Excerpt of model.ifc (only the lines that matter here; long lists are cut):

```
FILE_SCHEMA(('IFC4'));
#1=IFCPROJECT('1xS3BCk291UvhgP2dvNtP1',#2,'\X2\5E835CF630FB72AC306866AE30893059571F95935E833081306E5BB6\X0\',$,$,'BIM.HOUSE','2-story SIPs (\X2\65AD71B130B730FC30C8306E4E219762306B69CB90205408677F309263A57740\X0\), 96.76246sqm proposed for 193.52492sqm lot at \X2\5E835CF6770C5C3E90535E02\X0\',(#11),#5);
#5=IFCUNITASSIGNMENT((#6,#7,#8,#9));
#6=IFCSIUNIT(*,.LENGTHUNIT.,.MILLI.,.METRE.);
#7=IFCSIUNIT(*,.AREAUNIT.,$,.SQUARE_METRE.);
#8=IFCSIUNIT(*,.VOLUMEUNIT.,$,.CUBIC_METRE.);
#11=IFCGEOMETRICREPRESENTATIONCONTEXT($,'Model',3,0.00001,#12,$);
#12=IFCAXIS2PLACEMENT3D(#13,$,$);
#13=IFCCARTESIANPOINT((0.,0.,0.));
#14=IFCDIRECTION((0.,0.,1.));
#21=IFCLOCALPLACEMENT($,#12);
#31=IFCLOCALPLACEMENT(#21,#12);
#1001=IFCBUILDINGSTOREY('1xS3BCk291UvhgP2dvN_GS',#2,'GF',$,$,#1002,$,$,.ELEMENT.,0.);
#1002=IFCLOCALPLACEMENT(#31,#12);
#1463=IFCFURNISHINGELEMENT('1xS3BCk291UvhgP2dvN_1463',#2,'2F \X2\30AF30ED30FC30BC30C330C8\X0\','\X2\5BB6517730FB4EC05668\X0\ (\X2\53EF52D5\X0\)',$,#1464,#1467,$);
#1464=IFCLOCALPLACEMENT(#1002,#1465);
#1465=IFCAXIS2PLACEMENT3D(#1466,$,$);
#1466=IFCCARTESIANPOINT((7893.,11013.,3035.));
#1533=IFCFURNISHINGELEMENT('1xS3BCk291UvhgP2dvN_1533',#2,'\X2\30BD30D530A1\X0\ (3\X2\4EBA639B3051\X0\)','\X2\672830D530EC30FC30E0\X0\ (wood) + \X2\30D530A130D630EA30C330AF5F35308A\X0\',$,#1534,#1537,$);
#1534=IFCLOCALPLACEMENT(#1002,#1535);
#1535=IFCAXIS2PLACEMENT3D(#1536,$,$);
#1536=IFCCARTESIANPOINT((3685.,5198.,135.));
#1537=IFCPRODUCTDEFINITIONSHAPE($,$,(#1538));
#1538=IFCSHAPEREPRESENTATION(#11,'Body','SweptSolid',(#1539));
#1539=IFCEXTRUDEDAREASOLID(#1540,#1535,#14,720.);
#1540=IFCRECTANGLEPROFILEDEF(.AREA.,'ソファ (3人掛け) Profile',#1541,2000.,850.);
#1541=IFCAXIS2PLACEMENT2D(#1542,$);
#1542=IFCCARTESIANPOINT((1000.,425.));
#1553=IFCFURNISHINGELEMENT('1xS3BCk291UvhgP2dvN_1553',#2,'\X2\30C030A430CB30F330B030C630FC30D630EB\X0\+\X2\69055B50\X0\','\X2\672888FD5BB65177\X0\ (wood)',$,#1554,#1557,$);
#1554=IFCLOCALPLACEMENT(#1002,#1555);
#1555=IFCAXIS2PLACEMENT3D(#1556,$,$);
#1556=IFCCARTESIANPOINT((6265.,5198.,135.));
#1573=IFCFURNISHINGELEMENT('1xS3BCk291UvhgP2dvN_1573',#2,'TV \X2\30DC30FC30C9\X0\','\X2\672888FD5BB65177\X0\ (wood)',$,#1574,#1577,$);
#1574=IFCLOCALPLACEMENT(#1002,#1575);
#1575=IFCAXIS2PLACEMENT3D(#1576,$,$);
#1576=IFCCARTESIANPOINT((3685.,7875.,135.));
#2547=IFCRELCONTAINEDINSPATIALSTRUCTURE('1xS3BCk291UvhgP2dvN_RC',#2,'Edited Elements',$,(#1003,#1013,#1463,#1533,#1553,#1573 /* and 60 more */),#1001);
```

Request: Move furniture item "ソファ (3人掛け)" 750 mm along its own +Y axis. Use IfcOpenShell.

```python
import ifcopenshell
import ifcopenshell.api.geometry
import ifcopenshell.util.placement

model = ifcopenshell.open("model.ifc")

item = model.by_id(1533)
matrix = ifcopenshell.util.placement.get_local_placement(item.ObjectPlacement)
matrix[:3, 3] += matrix[:3, 1] * 750.0
ifcopenshell.api.geometry.edit_object_placement(model, product=item, matrix=matrix, is_si=False)

print(ifcopenshell.util.placement.get_local_placement(item.ObjectPlacement).round(3) + 0.0)

model.write("model_v2.ifc")
```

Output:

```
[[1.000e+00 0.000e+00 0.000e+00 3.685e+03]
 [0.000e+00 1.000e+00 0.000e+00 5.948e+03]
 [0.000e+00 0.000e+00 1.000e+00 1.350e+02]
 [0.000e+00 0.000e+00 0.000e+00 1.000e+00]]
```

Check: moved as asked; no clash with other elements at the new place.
